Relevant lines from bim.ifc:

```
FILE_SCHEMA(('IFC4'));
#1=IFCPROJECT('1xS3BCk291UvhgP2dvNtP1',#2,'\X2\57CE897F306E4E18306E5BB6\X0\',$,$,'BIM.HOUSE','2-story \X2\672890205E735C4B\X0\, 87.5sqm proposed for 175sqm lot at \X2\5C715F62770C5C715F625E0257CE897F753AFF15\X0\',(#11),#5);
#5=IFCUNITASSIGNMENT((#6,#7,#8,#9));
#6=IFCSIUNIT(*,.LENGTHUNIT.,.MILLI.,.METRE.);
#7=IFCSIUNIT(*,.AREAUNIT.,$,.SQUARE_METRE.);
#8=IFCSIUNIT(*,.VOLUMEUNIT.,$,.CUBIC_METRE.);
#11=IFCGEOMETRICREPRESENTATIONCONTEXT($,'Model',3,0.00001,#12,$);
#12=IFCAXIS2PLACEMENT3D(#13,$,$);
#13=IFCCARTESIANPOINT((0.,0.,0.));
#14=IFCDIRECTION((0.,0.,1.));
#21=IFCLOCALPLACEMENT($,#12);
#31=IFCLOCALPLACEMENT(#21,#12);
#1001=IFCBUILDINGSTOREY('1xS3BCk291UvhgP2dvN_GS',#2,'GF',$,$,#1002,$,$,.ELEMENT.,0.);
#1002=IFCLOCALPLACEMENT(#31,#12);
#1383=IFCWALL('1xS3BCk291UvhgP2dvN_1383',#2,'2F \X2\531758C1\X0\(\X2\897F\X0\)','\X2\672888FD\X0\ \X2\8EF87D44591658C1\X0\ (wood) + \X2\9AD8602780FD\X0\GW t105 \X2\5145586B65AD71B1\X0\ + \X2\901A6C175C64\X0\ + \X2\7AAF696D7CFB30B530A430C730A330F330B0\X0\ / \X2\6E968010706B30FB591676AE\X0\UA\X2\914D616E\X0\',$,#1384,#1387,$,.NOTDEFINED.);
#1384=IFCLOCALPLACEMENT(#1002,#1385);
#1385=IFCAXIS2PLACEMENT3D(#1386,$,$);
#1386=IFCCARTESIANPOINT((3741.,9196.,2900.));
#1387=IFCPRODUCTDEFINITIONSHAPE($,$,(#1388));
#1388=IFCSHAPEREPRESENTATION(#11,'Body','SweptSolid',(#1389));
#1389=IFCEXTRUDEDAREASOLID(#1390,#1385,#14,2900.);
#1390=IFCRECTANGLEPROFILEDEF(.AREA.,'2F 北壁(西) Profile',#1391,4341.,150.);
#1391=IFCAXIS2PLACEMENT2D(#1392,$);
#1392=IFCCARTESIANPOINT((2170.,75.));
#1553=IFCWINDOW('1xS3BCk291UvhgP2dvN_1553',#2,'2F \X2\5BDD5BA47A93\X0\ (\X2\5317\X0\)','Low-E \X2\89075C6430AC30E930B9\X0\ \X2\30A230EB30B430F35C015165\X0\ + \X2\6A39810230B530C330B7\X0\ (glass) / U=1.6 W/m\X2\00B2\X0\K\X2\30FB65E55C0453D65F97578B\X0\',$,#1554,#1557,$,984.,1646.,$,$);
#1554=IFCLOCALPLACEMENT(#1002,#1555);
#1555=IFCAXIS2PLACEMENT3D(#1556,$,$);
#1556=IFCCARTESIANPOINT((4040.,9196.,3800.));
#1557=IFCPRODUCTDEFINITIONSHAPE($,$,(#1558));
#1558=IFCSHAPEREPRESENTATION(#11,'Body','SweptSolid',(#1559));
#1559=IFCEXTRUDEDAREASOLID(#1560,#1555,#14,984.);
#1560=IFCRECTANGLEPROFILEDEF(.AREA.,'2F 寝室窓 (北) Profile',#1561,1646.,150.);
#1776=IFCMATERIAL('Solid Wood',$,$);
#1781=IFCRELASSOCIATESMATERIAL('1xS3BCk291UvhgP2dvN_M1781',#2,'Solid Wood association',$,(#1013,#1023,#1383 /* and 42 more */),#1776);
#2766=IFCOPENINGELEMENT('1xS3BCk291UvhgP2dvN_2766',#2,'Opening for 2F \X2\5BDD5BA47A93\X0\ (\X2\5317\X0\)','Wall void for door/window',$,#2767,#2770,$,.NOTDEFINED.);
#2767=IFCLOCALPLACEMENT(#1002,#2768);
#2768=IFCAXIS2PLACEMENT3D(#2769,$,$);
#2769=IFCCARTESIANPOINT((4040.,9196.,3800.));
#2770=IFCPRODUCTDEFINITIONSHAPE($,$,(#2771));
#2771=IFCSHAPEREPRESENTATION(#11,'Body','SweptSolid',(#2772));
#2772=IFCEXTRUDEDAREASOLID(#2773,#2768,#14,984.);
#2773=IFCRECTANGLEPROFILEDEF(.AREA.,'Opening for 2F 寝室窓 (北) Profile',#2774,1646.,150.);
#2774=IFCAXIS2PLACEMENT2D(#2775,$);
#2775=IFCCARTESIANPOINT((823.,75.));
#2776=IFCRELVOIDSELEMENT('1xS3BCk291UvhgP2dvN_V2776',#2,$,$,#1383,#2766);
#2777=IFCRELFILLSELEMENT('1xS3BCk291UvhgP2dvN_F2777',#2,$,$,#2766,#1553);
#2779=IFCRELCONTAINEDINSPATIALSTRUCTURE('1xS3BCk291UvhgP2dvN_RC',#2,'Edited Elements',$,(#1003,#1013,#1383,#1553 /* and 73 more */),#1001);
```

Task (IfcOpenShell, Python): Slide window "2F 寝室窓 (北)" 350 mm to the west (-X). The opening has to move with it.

```python
import ifcopenshell
import ifcopenshell.api.geometry
import ifcopenshell.util.placement
import ifcopenshell.util.unit

model = ifcopenshell.open("bim.ifc")
unit_scale = ifcopenshell.util.unit.calculate_unit_scale(model)

window = model.by_guid("1xS3BCk291UvhgP2dvN_1553")
opening = window.FillsVoids[0].RelatingOpeningElement
wall = opening.VoidsElements[0].RelatingBuildingElement

wall_matrix = ifcopenshell.util.placement.get_local_placement(wall.ObjectPlacement)
shift = wall_matrix[:3, 0] * -0.35 / unit_scale
before = ifcopenshell.util.placement.get_local_placement(window.ObjectPlacement)[:3, 3].copy()

# The window is not placed relative to its opening, so move both.
for product in (opening, window):
    matrix = ifcopenshell.util.placement.get_local_placement(product.ObjectPlacement)
    matrix[:3, 3] += shift
    ifcopenshell.api.geometry.edit_object_placement(model, product=product, matrix=matrix, is_si=False)

after = ifcopenshell.util.placement.get_local_placement(window.ObjectPlacement)[:3, 3]
print("window moved by", (after - before).round(3) + 0.0)

model.write("bim_rev.ifc")
```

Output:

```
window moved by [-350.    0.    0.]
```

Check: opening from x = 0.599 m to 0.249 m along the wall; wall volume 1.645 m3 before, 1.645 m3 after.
